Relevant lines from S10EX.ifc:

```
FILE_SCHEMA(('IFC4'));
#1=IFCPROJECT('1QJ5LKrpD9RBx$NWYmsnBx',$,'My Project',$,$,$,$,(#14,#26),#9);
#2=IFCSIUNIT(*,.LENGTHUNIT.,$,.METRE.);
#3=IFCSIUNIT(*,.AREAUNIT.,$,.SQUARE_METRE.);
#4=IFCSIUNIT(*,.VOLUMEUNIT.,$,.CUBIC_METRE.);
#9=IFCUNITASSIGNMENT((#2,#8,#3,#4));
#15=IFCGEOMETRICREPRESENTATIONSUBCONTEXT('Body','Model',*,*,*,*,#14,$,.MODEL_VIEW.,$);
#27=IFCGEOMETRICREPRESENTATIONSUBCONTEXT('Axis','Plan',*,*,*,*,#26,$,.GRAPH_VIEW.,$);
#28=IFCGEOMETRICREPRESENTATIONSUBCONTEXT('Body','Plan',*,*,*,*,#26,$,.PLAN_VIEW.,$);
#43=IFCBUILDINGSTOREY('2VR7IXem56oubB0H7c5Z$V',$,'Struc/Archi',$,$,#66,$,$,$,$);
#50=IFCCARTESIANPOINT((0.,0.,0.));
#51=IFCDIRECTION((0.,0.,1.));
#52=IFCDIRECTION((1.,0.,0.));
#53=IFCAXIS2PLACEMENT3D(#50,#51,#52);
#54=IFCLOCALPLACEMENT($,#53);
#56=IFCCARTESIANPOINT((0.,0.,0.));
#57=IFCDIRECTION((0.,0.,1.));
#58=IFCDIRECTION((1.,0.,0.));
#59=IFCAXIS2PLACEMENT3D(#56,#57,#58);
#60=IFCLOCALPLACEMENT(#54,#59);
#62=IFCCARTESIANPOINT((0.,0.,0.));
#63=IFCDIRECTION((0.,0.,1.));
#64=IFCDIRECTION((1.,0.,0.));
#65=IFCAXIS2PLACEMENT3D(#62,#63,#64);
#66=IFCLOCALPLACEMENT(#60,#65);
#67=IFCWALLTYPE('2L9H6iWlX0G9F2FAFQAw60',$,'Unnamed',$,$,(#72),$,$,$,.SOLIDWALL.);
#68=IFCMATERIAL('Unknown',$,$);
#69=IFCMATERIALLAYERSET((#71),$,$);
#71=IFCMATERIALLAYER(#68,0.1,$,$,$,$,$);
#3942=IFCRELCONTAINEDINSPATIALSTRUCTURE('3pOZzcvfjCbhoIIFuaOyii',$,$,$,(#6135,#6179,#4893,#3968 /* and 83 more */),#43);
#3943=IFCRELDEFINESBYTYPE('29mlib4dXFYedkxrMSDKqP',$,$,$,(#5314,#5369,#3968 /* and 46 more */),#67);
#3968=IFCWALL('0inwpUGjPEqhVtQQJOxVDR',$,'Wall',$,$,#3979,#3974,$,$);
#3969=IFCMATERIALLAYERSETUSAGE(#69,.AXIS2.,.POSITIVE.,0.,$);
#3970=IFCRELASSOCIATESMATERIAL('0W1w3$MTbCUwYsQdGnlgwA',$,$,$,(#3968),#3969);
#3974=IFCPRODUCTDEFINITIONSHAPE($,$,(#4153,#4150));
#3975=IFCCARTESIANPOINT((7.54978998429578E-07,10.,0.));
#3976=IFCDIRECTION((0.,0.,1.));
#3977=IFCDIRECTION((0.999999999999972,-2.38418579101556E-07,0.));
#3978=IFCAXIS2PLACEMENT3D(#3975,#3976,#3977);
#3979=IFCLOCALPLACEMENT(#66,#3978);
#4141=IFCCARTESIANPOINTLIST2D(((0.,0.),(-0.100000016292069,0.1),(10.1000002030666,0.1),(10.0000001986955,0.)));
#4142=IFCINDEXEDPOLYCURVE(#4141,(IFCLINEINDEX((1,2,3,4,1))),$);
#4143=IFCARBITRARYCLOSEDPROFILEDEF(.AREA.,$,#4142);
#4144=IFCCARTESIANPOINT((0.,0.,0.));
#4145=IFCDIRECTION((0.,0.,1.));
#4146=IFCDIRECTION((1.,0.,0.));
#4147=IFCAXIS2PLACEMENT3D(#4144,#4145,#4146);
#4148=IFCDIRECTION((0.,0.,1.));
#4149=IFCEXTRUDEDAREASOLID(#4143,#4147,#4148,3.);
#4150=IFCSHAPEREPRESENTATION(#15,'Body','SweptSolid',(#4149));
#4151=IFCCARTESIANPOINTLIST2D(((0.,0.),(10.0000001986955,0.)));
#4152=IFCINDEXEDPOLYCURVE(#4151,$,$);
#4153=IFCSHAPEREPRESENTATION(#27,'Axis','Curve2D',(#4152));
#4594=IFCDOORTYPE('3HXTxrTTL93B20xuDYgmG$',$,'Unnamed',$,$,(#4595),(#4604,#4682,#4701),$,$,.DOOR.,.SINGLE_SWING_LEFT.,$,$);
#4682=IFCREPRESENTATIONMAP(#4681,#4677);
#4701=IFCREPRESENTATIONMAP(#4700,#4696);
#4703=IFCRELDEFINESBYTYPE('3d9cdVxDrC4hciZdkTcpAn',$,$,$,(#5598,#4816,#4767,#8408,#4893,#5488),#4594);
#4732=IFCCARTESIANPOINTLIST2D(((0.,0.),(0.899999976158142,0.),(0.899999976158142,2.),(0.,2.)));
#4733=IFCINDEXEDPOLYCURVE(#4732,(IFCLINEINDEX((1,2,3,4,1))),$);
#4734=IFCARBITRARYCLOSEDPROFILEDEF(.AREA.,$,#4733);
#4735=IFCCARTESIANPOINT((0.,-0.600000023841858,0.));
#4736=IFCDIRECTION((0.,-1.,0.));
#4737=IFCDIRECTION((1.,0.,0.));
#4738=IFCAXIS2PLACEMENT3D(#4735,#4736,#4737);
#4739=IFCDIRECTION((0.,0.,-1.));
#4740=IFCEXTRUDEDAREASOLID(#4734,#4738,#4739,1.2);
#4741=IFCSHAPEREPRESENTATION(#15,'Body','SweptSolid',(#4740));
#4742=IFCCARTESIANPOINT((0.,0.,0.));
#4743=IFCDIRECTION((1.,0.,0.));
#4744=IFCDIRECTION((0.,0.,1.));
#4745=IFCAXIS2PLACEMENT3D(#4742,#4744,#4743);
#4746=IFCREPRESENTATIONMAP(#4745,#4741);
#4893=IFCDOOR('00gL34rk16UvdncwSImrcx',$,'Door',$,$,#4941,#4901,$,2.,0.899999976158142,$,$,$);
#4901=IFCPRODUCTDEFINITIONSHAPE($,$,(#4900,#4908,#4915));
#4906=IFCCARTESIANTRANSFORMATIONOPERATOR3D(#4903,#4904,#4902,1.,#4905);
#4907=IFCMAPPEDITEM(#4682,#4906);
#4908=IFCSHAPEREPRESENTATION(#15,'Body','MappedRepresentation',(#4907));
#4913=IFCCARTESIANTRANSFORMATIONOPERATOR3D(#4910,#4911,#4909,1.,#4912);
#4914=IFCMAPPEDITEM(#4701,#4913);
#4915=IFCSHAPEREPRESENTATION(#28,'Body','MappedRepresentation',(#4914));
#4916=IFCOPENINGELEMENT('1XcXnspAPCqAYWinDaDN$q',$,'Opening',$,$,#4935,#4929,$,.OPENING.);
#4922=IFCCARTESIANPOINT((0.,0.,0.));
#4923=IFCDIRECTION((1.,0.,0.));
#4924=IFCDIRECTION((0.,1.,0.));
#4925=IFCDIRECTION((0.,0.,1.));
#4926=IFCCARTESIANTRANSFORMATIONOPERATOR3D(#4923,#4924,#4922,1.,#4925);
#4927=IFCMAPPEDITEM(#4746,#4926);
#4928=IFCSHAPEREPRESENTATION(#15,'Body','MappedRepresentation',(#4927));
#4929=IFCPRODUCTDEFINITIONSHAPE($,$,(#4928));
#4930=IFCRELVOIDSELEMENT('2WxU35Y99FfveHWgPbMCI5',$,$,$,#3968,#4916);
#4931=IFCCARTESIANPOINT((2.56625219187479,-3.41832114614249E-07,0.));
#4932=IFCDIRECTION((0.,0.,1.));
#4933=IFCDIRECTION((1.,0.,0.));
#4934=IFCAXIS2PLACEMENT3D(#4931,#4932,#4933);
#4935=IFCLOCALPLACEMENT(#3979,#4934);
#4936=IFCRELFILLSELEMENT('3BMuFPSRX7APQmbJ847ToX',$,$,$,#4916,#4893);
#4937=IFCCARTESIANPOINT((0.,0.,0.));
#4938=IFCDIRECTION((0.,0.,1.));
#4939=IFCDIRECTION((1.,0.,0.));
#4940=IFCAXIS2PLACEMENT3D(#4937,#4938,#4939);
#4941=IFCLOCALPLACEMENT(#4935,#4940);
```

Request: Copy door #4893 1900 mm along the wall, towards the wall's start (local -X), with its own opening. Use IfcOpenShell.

```python
import ifcopenshell
import ifcopenshell.api.feature
import ifcopenshell.api.geometry
import ifcopenshell.api.root
import ifcopenshell.geom
import ifcopenshell.util.element
import ifcopenshell.util.placement
import ifcopenshell.util.shape
import ifcopenshell.util.unit

model = ifcopenshell.open("S10EX.ifc")
unit_scale = ifcopenshell.util.unit.calculate_unit_scale(model)
settings = ifcopenshell.geom.settings()


def volume(element):
    """Net volume in cubic metres, openings subtracted."""
    shape = ifcopenshell.geom.create_shape(settings, element)
    return ifcopenshell.util.shape.get_volume(shape.geometry)


door = model.by_guid("00gL34rk16UvdncwSImrcx")
opening = door.FillsVoids[0].RelatingOpeningElement
wall = opening.VoidsElements[0].RelatingBuildingElement
before = volume(wall)
shift = ifcopenshell.util.placement.get_local_placement(wall.ObjectPlacement)[:3, 0] * -1.9 / unit_scale

# copy_class copies the void relationship, type, container and properties, but no geometry.
new_opening = ifcopenshell.api.root.copy_class(model, product=opening)
new_opening.Representation = ifcopenshell.util.element.copy_deep(
    model, opening.Representation, exclude=["IfcGeometricRepresentationContext", "IfcRepresentationMap"]
)
new_door = ifcopenshell.api.root.copy_class(model, product=door)
new_door.Representation = ifcopenshell.util.element.copy_deep(
    model, door.Representation, exclude=["IfcGeometricRepresentationContext", "IfcRepresentationMap"]
)
ifcopenshell.api.feature.add_filling(model, opening=new_opening, element=new_door)

for old, new in ((opening, new_opening), (door, new_door)):
    matrix = ifcopenshell.util.placement.get_local_placement(old.ObjectPlacement)
    matrix[:3, 3] += shift
    ifcopenshell.api.geometry.edit_object_placement(model, product=new, matrix=matrix, is_si=False)

after = volume(wall)

print(f"wall volume {before:.3f} -> {after:.3f} m3")

model.write("S10EX_updated.ifc")
```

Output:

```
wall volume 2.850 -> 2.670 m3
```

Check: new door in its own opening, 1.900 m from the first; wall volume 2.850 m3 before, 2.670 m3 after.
